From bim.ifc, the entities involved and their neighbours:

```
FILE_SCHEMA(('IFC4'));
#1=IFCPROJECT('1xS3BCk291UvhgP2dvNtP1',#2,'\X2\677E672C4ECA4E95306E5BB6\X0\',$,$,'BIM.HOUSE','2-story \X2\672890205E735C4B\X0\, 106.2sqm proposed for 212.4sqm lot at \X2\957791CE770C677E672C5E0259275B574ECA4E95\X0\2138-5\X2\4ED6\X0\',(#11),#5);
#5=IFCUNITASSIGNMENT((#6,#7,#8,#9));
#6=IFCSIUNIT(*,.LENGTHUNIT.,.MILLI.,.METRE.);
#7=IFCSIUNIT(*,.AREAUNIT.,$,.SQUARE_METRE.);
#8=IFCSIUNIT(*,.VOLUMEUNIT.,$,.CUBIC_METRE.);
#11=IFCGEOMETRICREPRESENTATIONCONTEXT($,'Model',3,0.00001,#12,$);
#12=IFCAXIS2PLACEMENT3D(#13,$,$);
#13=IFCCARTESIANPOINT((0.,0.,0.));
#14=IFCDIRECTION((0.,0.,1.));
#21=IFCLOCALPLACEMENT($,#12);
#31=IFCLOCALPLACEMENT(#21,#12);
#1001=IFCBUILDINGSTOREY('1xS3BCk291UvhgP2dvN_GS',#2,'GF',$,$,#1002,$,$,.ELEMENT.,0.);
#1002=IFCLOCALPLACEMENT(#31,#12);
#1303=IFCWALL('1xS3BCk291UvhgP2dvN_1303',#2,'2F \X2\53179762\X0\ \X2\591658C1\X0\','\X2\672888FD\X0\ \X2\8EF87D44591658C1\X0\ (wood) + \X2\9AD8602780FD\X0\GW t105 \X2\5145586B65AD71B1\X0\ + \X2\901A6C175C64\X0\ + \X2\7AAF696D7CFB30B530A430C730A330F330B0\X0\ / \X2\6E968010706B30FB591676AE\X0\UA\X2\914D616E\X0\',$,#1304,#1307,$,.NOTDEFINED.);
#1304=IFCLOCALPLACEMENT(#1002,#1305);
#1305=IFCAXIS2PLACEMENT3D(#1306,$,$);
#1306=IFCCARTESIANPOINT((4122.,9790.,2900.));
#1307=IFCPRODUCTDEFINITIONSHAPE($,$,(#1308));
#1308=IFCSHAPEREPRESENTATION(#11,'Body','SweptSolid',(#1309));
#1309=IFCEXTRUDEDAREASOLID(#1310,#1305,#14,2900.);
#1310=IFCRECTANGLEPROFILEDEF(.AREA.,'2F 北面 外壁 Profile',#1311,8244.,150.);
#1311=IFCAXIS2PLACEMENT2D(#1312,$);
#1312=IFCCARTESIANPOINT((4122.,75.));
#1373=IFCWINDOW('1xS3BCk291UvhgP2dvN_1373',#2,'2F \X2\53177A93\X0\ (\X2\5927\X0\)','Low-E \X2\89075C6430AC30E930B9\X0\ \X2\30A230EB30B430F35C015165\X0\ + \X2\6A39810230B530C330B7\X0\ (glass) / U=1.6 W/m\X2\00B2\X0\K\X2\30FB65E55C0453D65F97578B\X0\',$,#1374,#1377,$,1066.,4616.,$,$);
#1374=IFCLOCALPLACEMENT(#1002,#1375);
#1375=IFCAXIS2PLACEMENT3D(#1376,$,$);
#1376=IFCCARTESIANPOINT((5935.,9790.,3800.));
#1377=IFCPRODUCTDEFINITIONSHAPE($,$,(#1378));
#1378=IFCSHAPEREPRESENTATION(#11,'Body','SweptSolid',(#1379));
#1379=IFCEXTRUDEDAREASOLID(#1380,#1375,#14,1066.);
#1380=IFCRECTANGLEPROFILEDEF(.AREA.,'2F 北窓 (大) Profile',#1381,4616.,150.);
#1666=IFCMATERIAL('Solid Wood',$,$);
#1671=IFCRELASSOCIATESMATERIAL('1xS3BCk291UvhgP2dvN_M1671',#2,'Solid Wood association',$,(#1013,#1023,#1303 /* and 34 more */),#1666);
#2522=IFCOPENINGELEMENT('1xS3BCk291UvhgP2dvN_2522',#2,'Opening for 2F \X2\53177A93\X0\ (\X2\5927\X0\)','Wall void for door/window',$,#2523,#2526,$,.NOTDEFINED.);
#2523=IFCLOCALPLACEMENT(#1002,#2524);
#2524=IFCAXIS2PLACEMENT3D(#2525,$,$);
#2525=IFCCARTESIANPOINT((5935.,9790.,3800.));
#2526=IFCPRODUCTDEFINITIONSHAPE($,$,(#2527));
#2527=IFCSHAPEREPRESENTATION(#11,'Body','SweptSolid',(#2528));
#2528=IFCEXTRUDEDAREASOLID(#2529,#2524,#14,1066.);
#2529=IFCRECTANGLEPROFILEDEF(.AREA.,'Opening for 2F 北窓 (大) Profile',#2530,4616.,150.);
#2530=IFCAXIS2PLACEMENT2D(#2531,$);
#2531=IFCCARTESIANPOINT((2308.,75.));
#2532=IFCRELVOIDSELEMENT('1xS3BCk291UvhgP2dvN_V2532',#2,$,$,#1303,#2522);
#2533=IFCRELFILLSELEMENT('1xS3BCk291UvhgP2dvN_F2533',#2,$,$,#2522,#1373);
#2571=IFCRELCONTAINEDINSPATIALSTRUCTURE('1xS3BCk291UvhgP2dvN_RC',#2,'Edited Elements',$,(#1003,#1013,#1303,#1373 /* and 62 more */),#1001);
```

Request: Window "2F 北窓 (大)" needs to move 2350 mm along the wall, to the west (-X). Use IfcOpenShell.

```python
import ifcopenshell
import ifcopenshell.api.geometry
import ifcopenshell.util.placement
import ifcopenshell.util.unit

model = ifcopenshell.open("bim.ifc")
unit_scale = ifcopenshell.util.unit.calculate_unit_scale(model)

window = model.by_id(1373)
opening = window.FillsVoids[0].RelatingOpeningElement
wall = opening.VoidsElements[0].RelatingBuildingElement

wall_matrix = ifcopenshell.util.placement.get_local_placement(wall.ObjectPlacement)
shift = wall_matrix[:3, 0] * -2.35 / unit_scale
before = ifcopenshell.util.placement.get_local_placement(window.ObjectPlacement)[:3, 3].copy()

# The window is not placed relative to its opening, so move both.
for product in (opening, window):
    matrix = ifcopenshell.util.placement.get_local_placement(product.ObjectPlacement)
    matrix[:3, 3] += shift
    ifcopenshell.api.geometry.edit_object_placement(model, product=product, matrix=matrix, is_si=False)

after = ifcopenshell.util.placement.get_local_placement(window.ObjectPlacement)[:3, 3]
print("window moved by", (after - before).round(3) + 0.0)

model.write("bim_updated.ifc")
```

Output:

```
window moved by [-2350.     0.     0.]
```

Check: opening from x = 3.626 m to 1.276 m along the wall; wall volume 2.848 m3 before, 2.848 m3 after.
